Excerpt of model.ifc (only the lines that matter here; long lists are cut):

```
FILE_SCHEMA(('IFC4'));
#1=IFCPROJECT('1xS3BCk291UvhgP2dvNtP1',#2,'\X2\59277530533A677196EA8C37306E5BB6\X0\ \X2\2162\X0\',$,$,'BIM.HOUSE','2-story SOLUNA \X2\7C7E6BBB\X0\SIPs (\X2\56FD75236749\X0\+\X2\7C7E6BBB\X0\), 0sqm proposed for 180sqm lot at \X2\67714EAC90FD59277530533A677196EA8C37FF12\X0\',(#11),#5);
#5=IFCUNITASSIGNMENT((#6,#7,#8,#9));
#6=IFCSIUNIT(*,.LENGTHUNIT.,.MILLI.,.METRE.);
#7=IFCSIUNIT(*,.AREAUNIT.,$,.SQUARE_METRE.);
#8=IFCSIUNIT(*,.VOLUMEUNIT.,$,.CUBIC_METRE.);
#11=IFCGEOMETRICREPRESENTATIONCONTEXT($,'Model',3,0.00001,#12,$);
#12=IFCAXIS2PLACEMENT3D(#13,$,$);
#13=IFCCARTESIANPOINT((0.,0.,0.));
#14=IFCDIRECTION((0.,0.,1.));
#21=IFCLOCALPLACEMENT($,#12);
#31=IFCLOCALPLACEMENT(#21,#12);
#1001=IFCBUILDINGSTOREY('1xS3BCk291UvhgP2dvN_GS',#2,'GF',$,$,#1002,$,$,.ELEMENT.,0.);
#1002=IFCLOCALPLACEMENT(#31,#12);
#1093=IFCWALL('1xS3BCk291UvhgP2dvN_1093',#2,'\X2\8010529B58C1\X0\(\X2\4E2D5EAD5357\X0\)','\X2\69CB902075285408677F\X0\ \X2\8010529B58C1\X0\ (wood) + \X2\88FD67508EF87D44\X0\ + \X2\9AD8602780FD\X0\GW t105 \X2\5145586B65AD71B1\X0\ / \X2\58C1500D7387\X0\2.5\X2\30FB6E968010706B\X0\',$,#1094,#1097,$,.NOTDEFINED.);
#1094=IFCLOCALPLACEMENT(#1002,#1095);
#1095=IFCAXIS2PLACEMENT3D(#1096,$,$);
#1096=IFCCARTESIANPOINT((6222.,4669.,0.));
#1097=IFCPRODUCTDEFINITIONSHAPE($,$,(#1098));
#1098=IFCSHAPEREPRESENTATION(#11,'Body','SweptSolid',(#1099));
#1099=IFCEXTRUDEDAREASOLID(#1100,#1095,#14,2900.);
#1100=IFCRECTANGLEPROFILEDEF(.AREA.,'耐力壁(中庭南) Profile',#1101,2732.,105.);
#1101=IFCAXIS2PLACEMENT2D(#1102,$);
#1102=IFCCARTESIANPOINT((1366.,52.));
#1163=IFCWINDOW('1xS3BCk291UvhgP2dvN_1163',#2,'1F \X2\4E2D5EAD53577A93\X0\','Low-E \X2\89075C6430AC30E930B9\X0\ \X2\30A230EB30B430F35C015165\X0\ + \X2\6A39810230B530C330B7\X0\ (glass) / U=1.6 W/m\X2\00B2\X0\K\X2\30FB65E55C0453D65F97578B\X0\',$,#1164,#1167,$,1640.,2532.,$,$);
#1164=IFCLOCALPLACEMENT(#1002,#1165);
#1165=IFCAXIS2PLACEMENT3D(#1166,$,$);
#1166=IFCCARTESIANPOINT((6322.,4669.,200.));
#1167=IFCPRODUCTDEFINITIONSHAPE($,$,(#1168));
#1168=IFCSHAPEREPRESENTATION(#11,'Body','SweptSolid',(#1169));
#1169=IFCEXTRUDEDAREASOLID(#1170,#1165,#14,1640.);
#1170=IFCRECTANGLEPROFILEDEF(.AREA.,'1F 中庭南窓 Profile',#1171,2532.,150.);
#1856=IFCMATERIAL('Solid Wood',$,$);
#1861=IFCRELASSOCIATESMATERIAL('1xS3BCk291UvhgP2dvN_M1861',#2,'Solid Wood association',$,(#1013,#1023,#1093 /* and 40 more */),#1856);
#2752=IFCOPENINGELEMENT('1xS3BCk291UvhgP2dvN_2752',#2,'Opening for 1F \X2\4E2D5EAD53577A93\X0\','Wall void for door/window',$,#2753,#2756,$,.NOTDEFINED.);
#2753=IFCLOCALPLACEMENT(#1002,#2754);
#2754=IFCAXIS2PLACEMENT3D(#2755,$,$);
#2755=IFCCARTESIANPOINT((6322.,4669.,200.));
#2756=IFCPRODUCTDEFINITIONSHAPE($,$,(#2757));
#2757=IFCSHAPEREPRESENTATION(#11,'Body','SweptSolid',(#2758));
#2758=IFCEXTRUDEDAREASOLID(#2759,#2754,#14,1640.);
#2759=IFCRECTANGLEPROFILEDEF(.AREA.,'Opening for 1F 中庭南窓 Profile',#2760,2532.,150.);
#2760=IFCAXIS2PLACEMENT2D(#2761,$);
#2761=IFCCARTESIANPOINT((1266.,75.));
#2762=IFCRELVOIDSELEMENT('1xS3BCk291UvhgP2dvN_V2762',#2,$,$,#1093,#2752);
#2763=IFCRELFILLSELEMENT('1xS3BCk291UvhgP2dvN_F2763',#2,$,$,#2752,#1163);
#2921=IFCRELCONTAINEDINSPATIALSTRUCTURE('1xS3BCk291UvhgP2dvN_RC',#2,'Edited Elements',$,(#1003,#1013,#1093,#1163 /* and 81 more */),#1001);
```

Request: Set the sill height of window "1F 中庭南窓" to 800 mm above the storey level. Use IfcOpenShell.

```python
import numpy as np
import ifcopenshell
import ifcopenshell.api.geometry
import ifcopenshell.geom
import ifcopenshell.util.element
import ifcopenshell.util.placement
import ifcopenshell.util.shape
import ifcopenshell.util.unit

model = ifcopenshell.open("model.ifc")
unit_scale = ifcopenshell.util.unit.calculate_unit_scale(model)

window = model.by_guid("1xS3BCk291UvhgP2dvN_1163")
opening = window.FillsVoids[0].RelatingOpeningElement
storey = ifcopenshell.util.element.get_container(window, ifc_class="IfcBuildingStorey")
level = ifcopenshell.util.placement.get_local_placement(storey.ObjectPlacement)[2, 3]

# The opening's origin need not be at the sill, so measure its lowest point.
shape = ifcopenshell.geom.create_shape(ifcopenshell.geom.settings(), opening)
bottom = ifcopenshell.util.shape.get_shape_bottom_elevation(shape, shape.geometry) / unit_scale
dz = level + 800.0 - bottom

shift = np.array([0.0, 0.0, dz])
# The window is not placed relative to its opening, so move both.
for product in (opening, window):
    matrix = ifcopenshell.util.placement.get_local_placement(product.ObjectPlacement)
    matrix[:3, 3] += shift
    ifcopenshell.api.geometry.edit_object_placement(model, product=product, matrix=matrix, is_si=False)

print(f"moved by {dz * unit_scale:+.3f} m")

model.write("model_updated.ifc")
```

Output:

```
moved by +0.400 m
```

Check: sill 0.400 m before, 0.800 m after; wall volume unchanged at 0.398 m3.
